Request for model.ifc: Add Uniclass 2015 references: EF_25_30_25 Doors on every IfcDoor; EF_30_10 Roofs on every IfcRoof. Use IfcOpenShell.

First a look at what the model holds.

```python
import ifcopenshell

model = ifcopenshell.open("model.ifc")
print(model.schema)
print("classifications:", [c.Name for c in model.by_type("IfcClassification")])
for ifc_class in ("IfcDoor", "IfcRoof", "IfcStair", "IfcWall", "IfcWindow"):
    print(ifc_class, len(model.by_type(ifc_class)))
```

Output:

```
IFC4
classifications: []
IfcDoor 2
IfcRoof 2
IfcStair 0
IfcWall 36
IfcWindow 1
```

```python
import ifcopenshell
import ifcopenshell.api.classification

model = ifcopenshell.open("model.ifc")

system = ifcopenshell.api.classification.add_classification(model, classification="Uniclass 2015")

codes = {
    "IfcDoor": ("EF_25_30_25", "Doors"),
    "IfcRoof": ("EF_30_10", "Roofs"),
}
for ifc_class, (code, name) in codes.items():
    products = model.by_type(ifc_class)
    ifcopenshell.api.classification.add_reference(
        model, products=products, classification=system, identification=code, name=name
    )
    print(code, len(products))

model.write("model_rev.ifc")
```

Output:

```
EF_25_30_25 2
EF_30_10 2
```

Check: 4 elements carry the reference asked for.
